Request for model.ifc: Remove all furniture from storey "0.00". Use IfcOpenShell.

First a look at what the model holds.

```python
import ifcopenshell
import ifcopenshell.util.element

model = ifcopenshell.open("model.ifc")
print(model.schema)
storey = next(s for s in model.by_type("IfcBuildingStorey") if s.Name == "0.00")
furniture = [e for e in ifcopenshell.util.element.get_decomposition(storey) if e.is_a("IfcFurnishingElement")]
seen = {}
for e in furniture:
    element_type = ifcopenshell.util.element.get_type(e)
    name = element_type.Name if element_type not in (None, e) else None
    seen[name] = seen.get(name, 0) + 1
for name, count in sorted(seen.items(), key=str):
    print(count, "x", name)
```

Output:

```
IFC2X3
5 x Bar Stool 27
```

```python
import ifcopenshell
import ifcopenshell.api.root
import ifcopenshell.util.element

model = ifcopenshell.open("model.ifc")

storey = next(s for s in model.by_type("IfcBuildingStorey") if s.Name == "0.00")
furniture = [e for e in ifcopenshell.util.element.get_decomposition(storey) if e.is_a("IfcFurnishingElement")]

for e in furniture:
    ifcopenshell.api.root.remove_product(model, product=e)
print(len(furniture), "removed")

model.write("model_v2.ifc")
```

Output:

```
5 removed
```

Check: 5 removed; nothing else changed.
